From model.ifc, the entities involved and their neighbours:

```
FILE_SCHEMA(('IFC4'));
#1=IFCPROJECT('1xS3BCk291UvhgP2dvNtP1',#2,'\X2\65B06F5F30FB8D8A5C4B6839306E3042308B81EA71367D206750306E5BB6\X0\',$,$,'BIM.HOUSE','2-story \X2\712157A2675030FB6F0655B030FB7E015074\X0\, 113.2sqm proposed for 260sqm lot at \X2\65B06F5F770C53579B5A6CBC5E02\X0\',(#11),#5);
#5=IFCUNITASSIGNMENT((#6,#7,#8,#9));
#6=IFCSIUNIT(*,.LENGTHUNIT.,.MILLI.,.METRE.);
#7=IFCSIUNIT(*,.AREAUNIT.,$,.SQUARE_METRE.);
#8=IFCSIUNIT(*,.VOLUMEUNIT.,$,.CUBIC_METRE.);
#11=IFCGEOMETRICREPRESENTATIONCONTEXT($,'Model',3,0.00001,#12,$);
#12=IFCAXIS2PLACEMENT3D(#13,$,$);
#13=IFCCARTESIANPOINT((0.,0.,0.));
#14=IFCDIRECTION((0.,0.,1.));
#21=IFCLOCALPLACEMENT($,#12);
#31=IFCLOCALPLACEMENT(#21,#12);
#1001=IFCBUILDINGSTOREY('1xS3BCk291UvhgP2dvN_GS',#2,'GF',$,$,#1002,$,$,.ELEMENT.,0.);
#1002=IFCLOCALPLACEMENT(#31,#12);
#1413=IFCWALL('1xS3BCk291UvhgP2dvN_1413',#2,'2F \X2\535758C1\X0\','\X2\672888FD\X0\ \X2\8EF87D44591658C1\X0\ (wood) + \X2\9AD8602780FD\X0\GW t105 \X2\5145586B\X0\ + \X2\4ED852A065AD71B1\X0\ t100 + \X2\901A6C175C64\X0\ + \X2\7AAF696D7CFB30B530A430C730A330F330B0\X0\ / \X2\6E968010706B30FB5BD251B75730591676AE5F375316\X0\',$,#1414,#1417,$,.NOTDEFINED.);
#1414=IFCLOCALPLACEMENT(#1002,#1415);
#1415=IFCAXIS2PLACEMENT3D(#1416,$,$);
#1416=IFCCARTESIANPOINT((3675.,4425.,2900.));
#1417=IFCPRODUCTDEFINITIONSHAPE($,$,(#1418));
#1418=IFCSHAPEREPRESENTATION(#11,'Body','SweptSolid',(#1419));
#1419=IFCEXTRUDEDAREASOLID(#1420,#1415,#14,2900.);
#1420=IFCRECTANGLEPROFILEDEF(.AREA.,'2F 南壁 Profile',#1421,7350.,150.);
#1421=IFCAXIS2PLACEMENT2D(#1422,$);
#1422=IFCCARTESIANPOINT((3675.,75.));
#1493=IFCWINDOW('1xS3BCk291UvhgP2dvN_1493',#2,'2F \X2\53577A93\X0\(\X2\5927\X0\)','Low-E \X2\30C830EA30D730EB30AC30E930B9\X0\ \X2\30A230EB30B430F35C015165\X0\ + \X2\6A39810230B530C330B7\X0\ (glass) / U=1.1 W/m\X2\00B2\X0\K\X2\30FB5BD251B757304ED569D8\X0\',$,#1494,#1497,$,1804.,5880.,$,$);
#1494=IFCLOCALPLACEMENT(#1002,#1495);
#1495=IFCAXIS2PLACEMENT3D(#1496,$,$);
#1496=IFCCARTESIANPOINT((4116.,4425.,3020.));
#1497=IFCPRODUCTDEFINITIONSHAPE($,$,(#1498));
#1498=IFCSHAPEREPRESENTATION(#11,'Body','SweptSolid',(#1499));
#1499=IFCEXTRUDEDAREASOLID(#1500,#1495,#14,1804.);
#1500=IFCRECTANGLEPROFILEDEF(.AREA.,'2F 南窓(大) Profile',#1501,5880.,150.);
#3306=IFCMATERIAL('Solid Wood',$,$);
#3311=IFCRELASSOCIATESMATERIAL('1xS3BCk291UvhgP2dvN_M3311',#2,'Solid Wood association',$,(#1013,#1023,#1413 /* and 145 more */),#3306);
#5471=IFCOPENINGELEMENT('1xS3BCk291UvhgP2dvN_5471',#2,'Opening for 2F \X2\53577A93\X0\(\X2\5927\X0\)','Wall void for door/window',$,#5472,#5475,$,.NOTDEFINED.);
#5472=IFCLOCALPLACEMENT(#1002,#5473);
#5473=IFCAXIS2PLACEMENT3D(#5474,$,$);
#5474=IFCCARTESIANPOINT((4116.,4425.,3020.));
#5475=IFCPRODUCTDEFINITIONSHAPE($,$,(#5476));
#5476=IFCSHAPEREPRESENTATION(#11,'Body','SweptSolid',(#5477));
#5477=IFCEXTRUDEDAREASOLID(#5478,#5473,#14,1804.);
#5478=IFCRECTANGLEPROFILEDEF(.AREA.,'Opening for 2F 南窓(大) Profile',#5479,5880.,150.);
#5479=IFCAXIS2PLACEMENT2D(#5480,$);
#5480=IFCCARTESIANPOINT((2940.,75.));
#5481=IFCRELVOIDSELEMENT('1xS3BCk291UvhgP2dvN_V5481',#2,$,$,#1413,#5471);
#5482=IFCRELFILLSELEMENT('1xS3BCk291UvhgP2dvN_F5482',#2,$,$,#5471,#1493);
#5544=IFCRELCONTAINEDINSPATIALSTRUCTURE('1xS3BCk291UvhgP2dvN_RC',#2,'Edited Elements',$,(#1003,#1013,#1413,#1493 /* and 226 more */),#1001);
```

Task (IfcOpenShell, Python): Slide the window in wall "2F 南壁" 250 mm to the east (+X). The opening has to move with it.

```python
import ifcopenshell
import ifcopenshell.api.geometry
import ifcopenshell.util.placement

model = ifcopenshell.open("model.ifc")

window = model.by_guid("1xS3BCk291UvhgP2dvN_1493")
opening = window.FillsVoids[0].RelatingOpeningElement
wall = opening.VoidsElements[0].RelatingBuildingElement

wall_matrix = ifcopenshell.util.placement.get_local_placement(wall.ObjectPlacement)
shift = wall_matrix[:3, 0] * 250.0
before = ifcopenshell.util.placement.get_local_placement(window.ObjectPlacement)[:3, 3].copy()

# The window is not placed relative to its opening, so move both.
for product in (opening, window):
    matrix = ifcopenshell.util.placement.get_local_placement(product.ObjectPlacement)
    matrix[:3, 3] += shift
    ifcopenshell.api.geometry.edit_object_placement(model, product=product, matrix=matrix, is_si=False)

after = ifcopenshell.util.placement.get_local_placement(window.ObjectPlacement)[:3, 3]
print("window moved by", (after - before).round(3) + 0.0)

model.write("model_v2.ifc")
```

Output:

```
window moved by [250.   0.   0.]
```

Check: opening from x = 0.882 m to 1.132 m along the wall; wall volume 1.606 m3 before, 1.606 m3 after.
